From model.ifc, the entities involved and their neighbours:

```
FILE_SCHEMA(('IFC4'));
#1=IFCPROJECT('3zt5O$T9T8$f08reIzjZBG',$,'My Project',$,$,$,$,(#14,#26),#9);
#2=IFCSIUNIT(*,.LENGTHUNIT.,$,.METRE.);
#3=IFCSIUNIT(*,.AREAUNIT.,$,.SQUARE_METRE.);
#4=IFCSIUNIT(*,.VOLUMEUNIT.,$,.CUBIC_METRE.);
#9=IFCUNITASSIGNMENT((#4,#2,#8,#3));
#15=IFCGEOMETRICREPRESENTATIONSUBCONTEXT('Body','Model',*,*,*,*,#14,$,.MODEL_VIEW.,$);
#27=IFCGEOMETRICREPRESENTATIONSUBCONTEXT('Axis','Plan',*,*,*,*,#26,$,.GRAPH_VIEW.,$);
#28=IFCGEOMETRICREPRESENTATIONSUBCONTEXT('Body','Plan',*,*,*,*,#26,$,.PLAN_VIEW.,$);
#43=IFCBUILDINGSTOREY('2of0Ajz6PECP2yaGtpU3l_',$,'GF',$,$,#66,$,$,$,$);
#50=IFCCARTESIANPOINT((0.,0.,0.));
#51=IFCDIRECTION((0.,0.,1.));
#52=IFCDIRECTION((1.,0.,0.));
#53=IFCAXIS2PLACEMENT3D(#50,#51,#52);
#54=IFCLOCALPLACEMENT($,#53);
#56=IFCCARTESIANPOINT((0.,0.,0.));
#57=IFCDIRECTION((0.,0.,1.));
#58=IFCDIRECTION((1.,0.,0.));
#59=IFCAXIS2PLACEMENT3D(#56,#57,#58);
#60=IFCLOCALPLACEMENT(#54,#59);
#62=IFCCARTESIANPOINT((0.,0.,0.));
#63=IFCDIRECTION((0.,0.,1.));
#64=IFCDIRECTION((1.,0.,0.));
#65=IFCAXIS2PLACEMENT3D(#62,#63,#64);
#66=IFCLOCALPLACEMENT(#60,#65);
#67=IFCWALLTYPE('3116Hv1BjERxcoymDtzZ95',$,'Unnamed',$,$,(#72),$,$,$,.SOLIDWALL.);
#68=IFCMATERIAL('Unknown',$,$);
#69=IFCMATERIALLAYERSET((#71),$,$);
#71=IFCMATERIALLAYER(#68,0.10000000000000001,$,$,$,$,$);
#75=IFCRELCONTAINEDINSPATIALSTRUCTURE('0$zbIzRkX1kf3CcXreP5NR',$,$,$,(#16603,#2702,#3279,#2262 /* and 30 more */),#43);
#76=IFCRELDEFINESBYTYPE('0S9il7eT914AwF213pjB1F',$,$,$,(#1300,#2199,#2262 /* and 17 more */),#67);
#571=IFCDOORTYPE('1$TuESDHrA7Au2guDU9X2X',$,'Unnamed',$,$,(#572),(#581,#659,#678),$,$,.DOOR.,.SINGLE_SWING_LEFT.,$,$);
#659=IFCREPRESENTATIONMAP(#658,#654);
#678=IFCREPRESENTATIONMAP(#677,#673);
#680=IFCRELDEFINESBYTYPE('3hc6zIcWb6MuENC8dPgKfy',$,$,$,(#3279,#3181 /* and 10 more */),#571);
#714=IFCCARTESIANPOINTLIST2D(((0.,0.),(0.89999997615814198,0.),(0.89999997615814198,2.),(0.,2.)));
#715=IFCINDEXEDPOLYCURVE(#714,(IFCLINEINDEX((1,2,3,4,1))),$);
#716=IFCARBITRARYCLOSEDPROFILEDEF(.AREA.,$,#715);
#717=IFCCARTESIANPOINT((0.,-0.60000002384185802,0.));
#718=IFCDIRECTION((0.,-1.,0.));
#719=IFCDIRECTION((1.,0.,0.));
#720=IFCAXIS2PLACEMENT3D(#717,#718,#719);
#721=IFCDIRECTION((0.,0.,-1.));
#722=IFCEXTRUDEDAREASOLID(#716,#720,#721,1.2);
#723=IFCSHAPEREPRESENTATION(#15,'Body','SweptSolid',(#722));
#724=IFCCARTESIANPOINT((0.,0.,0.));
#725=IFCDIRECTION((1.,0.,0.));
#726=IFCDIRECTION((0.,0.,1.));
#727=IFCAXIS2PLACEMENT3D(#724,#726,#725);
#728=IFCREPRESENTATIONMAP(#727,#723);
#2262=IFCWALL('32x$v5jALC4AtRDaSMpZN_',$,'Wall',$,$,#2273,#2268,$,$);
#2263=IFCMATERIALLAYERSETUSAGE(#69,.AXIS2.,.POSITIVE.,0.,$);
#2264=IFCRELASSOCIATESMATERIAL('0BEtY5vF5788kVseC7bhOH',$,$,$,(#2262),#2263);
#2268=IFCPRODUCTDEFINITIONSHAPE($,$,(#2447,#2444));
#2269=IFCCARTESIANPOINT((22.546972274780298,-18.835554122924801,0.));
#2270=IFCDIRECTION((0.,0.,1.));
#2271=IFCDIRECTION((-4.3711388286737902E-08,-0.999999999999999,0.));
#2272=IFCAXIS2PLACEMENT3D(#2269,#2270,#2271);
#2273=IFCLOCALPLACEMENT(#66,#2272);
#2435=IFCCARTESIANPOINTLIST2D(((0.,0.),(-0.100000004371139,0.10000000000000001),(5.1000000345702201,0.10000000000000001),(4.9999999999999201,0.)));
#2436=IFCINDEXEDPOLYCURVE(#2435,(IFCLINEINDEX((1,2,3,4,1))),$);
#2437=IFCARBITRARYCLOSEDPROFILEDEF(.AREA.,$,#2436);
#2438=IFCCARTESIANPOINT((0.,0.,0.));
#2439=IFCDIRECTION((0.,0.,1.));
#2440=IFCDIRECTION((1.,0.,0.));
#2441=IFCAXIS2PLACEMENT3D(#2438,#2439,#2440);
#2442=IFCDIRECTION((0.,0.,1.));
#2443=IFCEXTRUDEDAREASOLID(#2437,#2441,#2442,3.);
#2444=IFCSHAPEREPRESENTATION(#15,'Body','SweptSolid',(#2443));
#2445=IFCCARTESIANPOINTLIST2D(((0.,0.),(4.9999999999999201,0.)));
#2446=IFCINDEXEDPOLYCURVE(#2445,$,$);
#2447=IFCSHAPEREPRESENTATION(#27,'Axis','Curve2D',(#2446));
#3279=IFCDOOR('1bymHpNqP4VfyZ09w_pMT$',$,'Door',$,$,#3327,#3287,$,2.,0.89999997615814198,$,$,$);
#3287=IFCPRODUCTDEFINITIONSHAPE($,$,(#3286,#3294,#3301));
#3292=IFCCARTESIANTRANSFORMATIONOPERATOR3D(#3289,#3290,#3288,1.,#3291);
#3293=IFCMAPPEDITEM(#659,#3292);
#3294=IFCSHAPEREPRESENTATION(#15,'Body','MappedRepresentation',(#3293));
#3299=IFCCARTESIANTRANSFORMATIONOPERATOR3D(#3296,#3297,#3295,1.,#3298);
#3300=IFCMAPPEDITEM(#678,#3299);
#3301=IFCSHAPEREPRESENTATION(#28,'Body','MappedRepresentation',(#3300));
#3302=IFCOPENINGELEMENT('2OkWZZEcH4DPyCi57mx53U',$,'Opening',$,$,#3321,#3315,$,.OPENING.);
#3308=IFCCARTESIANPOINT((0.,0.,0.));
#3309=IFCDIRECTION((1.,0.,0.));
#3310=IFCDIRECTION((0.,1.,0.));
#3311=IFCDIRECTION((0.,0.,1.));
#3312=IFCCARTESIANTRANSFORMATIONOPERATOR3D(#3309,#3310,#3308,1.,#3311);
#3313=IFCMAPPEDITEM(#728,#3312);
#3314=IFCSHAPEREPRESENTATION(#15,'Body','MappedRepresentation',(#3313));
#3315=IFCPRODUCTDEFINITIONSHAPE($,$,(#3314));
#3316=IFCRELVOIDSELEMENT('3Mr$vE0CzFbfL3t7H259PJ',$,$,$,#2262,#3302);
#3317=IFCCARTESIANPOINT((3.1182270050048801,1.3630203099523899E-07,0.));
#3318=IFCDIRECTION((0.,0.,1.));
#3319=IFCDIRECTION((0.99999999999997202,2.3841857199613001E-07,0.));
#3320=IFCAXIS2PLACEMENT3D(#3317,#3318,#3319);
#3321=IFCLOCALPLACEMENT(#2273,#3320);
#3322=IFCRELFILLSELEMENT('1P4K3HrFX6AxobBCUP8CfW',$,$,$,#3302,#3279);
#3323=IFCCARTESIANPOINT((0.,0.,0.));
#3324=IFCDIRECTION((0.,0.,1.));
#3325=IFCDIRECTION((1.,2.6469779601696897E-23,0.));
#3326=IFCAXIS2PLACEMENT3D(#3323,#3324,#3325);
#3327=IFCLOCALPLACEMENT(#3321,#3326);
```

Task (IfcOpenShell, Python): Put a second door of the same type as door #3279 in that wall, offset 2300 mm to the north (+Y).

```python
import ifcopenshell
import ifcopenshell.api.feature
import ifcopenshell.api.geometry
import ifcopenshell.api.root
import ifcopenshell.geom
import ifcopenshell.util.element
import ifcopenshell.util.placement
import ifcopenshell.util.shape
import ifcopenshell.util.unit

model = ifcopenshell.open("model.ifc")
unit_scale = ifcopenshell.util.unit.calculate_unit_scale(model)
settings = ifcopenshell.geom.settings()


def volume(element):
    """Net volume in cubic metres, openings subtracted."""
    shape = ifcopenshell.geom.create_shape(settings, element)
    return ifcopenshell.util.shape.get_volume(shape.geometry)


door = model.by_guid("1bymHpNqP4VfyZ09w_pMT$")
opening = door.FillsVoids[0].RelatingOpeningElement
wall = opening.VoidsElements[0].RelatingBuildingElement
before = volume(wall)
shift = ifcopenshell.util.placement.get_local_placement(wall.ObjectPlacement)[:3, 0] * -2.3 / unit_scale

# copy_class copies the void relationship, type, container and properties, but no geometry.
new_opening = ifcopenshell.api.root.copy_class(model, product=opening)
new_opening.Representation = ifcopenshell.util.element.copy_deep(
    model, opening.Representation, exclude=["IfcGeometricRepresentationContext", "IfcRepresentationMap"]
)
new_door = ifcopenshell.api.root.copy_class(model, product=door)
new_door.Representation = ifcopenshell.util.element.copy_deep(
    model, door.Representation, exclude=["IfcGeometricRepresentationContext", "IfcRepresentationMap"]
)
ifcopenshell.api.feature.add_filling(model, opening=new_opening, element=new_door)

for old, new in ((opening, new_opening), (door, new_door)):
    matrix = ifcopenshell.util.placement.get_local_placement(old.ObjectPlacement)
    matrix[:3, 3] += shift
    ifcopenshell.api.geometry.edit_object_placement(model, product=new, matrix=matrix, is_si=False)

after = volume(wall)

print(f"wall volume {before:.3f} -> {after:.3f} m3")

model.write("model-out.ifc")
```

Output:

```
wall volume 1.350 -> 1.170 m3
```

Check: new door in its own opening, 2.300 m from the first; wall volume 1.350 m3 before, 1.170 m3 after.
